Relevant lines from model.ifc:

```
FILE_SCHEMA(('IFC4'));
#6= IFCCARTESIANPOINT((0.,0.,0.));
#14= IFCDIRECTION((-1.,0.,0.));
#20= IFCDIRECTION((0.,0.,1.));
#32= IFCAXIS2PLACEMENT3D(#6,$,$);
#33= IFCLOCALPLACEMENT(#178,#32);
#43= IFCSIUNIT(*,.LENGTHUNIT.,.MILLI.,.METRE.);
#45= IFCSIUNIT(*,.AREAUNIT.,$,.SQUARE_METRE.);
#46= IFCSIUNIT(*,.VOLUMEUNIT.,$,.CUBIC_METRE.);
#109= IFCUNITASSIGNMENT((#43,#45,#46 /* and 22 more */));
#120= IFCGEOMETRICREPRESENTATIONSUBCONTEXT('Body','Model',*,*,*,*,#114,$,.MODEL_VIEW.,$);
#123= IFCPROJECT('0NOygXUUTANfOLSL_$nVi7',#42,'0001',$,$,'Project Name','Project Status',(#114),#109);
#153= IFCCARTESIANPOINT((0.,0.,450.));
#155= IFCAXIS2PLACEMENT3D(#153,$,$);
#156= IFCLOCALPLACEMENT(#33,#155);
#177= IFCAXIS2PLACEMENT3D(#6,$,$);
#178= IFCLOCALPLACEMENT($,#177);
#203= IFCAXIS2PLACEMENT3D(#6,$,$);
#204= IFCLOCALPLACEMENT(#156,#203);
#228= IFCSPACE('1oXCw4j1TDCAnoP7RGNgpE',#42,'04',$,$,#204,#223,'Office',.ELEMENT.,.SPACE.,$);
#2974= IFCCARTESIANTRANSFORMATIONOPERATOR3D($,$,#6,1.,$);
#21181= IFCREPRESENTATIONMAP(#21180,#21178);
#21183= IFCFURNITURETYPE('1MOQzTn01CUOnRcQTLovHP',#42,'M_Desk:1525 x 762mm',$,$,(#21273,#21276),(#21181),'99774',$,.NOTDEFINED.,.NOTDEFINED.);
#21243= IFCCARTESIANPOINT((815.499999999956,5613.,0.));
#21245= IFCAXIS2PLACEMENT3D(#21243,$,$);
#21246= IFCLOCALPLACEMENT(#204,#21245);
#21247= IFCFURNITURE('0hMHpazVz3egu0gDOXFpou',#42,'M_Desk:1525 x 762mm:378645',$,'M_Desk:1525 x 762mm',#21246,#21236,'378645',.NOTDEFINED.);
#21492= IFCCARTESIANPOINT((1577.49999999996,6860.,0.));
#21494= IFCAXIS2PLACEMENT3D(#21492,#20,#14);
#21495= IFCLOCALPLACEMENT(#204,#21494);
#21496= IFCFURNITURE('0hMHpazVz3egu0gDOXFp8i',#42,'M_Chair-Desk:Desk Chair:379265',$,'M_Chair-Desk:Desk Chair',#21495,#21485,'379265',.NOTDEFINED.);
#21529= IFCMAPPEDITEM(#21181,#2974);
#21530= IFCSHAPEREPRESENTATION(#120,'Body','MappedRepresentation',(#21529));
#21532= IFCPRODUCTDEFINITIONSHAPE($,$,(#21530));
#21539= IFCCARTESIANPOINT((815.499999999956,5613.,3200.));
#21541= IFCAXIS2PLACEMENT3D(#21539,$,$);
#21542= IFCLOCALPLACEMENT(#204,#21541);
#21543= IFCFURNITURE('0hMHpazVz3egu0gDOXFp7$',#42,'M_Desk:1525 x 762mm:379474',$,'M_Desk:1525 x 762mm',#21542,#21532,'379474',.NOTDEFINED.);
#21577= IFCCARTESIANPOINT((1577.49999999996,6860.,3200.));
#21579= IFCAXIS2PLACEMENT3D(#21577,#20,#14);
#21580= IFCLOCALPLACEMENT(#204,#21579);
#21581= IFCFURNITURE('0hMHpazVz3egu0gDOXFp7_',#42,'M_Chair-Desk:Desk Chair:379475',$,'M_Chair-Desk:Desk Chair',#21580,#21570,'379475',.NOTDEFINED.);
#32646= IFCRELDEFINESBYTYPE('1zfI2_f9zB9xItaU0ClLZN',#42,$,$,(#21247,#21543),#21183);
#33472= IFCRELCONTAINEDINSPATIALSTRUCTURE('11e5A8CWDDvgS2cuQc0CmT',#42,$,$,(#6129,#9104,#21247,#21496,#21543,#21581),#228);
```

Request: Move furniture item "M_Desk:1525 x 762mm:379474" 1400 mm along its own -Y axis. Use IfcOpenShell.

```python
import ifcopenshell
import ifcopenshell.api.geometry
import ifcopenshell.util.placement
import ifcopenshell.util.unit

model = ifcopenshell.open("model.ifc")
unit_scale = ifcopenshell.util.unit.calculate_unit_scale(model)

item = model.by_id(21543)
matrix = ifcopenshell.util.placement.get_local_placement(item.ObjectPlacement)
matrix[:3, 3] -= matrix[:3, 1] * 1.4 / unit_scale
ifcopenshell.api.geometry.edit_object_placement(model, product=item, matrix=matrix, is_si=False)

print(ifcopenshell.util.placement.get_local_placement(item.ObjectPlacement).round(3) + 0.0)

model.write("model-out.ifc")
```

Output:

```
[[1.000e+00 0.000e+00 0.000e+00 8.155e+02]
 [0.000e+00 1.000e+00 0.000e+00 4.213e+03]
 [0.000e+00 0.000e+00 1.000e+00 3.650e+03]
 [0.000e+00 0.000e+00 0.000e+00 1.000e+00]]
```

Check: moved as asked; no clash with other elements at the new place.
